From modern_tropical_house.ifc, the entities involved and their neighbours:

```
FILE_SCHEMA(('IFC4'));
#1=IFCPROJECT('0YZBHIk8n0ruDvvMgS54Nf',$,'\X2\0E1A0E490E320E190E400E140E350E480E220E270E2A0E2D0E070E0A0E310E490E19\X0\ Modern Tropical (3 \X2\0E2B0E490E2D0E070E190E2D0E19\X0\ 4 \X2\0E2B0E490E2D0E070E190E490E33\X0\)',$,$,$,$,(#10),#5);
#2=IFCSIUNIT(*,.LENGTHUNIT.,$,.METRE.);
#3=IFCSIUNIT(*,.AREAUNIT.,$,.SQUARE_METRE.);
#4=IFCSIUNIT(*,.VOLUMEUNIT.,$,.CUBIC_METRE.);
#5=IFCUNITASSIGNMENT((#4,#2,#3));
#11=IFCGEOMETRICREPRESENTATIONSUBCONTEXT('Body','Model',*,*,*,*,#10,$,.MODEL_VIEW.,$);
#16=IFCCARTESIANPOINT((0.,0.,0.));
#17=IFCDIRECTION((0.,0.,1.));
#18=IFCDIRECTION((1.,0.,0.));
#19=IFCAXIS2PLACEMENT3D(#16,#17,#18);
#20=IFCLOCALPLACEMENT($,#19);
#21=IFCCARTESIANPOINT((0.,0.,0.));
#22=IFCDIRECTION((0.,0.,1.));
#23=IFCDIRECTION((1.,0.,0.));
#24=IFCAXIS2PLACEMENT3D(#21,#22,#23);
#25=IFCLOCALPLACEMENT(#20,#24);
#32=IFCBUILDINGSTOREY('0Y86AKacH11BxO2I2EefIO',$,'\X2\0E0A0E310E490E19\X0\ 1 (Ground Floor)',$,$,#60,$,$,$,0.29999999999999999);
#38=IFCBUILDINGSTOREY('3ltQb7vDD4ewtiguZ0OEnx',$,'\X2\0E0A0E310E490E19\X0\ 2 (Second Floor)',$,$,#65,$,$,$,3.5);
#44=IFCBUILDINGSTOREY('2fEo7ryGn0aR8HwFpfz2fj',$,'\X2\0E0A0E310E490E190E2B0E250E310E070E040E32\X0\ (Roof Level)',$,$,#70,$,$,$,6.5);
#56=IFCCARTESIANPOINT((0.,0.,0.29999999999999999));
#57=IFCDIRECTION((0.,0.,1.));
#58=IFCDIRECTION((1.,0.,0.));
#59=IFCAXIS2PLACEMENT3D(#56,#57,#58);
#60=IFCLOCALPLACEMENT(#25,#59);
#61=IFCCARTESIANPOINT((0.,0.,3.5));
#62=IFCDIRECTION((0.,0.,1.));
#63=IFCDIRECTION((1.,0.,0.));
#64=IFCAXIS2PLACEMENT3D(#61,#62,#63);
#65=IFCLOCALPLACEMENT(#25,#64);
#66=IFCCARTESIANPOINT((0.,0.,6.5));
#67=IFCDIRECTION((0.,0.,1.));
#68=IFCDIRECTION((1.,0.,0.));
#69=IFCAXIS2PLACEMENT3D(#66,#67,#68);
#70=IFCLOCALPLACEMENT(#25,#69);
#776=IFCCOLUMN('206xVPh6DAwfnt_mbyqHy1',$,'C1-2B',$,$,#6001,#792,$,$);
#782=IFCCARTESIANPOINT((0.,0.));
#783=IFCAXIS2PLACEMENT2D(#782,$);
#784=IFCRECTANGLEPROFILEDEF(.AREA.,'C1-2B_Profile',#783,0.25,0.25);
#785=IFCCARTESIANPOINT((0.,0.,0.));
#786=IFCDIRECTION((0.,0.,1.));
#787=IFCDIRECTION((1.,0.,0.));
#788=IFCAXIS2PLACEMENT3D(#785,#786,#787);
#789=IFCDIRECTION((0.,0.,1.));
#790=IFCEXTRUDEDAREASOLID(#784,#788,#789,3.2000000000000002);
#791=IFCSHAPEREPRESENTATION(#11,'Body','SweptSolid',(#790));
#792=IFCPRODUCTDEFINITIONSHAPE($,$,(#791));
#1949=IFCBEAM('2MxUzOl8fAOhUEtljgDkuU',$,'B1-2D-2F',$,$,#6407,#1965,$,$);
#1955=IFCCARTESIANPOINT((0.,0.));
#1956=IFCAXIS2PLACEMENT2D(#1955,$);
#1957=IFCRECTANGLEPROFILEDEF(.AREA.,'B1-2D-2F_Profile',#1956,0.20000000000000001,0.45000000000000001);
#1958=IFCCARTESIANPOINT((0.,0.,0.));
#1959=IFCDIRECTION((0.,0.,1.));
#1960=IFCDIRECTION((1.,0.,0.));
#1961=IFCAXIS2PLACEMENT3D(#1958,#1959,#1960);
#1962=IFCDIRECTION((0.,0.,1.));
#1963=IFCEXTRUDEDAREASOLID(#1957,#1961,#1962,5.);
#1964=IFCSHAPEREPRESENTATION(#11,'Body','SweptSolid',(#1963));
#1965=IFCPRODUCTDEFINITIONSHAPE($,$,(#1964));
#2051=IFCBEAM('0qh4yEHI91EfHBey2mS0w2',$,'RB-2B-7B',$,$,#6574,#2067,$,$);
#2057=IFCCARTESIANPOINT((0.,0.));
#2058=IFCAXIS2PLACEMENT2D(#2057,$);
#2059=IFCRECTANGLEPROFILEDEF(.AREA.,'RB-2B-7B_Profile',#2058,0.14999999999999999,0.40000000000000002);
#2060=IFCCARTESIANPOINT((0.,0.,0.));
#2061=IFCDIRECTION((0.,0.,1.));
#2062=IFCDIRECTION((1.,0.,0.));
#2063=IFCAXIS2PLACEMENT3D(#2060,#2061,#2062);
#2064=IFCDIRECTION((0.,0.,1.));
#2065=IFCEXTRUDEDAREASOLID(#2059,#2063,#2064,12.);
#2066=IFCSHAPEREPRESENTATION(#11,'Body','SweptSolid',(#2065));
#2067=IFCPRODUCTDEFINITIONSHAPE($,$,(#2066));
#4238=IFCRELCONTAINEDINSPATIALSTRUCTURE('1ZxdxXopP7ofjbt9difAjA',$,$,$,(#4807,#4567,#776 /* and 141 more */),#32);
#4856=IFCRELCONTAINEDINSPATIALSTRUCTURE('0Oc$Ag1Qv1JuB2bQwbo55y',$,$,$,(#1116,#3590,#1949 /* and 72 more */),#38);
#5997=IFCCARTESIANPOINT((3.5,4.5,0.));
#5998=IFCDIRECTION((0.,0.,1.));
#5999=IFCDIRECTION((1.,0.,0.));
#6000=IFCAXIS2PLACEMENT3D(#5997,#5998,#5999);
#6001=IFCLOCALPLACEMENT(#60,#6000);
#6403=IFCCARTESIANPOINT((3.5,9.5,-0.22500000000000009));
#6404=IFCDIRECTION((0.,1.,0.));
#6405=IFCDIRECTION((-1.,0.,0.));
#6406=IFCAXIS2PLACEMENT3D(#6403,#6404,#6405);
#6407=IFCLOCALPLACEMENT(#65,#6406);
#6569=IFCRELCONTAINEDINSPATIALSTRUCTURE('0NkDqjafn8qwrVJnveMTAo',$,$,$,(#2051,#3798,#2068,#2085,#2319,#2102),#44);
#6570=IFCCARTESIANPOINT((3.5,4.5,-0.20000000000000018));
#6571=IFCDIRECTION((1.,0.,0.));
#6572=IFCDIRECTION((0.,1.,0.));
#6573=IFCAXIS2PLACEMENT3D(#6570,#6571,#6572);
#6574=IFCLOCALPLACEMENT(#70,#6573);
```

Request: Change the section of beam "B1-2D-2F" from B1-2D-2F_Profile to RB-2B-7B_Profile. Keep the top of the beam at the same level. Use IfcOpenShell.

```python
import ifcopenshell
import ifcopenshell.util.element
import ifcopenshell.util.representation

model = ifcopenshell.open("modern_tropical_house.ifc")

member = model.by_guid("2MxUzOl8fAOhUEtljgDkuU")
source = next(p for p in model.by_type("IfcRectangleProfileDef") if p.ProfileName == "RB-2B-7B_Profile")

body = ifcopenshell.util.representation.get_representation(member, "Model", "Body")
solid = body.Items[0]
old_profile = solid.SweptArea

# Copy the section's sizes but keep this member's own profile position.
profile = ifcopenshell.util.element.copy(model, source)
# Profiles are centred, so shift by half the change in depth to hold the top.
shift = (old_profile.YDim - profile.YDim) / 2
x, y = old_profile.Position.Location.Coordinates
up = (0.0, 1.0)  # upwards, in the solid's own plane
location = model.createIfcCartesianPoint((x + up[0] * shift, y + up[1] * shift))
profile.Position = model.createIfcAxis2Placement2D(location, old_profile.Position.RefDirection)
solid.SweptArea = profile
if not model.get_total_inverses(old_profile):
    ifcopenshell.util.element.remove_deep2(model, old_profile)

print(solid.SweptArea)

model.write("modern_tropical_house_edited.ifc")
```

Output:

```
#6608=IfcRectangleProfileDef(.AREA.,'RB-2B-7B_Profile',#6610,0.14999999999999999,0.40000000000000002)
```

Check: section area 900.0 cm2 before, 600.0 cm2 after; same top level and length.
